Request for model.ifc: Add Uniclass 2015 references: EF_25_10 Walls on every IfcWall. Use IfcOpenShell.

First a look at what the model holds.

```python
import ifcopenshell

model = ifcopenshell.open("model.ifc")
print(model.schema)
print("classifications:", [c.Name for c in model.by_type("IfcClassification")])
for ifc_class in ("IfcDoor", "IfcRoof", "IfcStair", "IfcWall", "IfcWindow"):
    print(ifc_class, len(model.by_type(ifc_class)))
```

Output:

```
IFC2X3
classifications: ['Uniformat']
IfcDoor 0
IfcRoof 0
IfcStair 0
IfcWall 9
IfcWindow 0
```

```python
import ifcopenshell
import ifcopenshell.api.classification

model = ifcopenshell.open("model.ifc")

# IFC2X3 requires Source and Edition and has no link from the project to the system.
system = model.create_entity("IfcClassification", Source="NBS", Edition="2015", Name="Uniclass 2015")

codes = {
    "IfcWall": ("EF_25_10", "Walls"),
}
for ifc_class, (code, name) in codes.items():
    products = model.by_type(ifc_class)
    ifcopenshell.api.classification.add_reference(
        model, products=products, classification=system, identification=code, name=name
    )
    print(code, len(products))

model.write("model-out.ifc")
```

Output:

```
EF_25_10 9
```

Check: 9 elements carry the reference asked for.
